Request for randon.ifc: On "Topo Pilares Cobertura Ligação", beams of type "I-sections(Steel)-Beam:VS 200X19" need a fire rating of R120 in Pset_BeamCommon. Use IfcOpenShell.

First a look at what the model holds.

```python
import ifcopenshell
import ifcopenshell.util.element

model = ifcopenshell.open("randon.ifc")
print(model.schema)
storey = next(s for s in model.by_type("IfcBuildingStorey") if s.Name == "Topo Pilares Cobertura Ligação")
beams = [e for e in ifcopenshell.util.element.get_decomposition(storey) if e.is_a("IfcBeam")]
seen = {}
for e in beams:
    element_type = ifcopenshell.util.element.get_type(e)
    key = (element_type.Name if element_type != e and element_type else None, ifcopenshell.util.element.get_pset(e, "Pset_BeamCommon", "FireRating"))
    seen[key] = seen.get(key, 0) + 1
for (name, value), count in sorted(seen.items(), key=str):
    print(count, "x", name, "|", value)
```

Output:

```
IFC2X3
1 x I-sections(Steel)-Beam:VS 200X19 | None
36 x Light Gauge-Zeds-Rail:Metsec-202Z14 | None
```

```python
import ifcopenshell
import ifcopenshell.api.pset
import ifcopenshell.util.element

model = ifcopenshell.open("randon.ifc")

storey = next(s for s in model.by_type("IfcBuildingStorey") if s.Name == "Topo Pilares Cobertura Ligação")
beams = [e for e in ifcopenshell.util.element.get_decomposition(storey) if e.is_a("IfcBeam")]

count = 0
for e in beams:
    element_type = ifcopenshell.util.element.get_type(e)
    if element_type in (None, e) or element_type.Name != "I-sections(Steel)-Beam:VS 200X19":
        continue
    # add_pset returns the element's existing set when there is one.
    pset = ifcopenshell.api.pset.add_pset(model, product=e, name="Pset_BeamCommon")
    ifcopenshell.api.pset.edit_pset(model, pset=pset, properties={"FireRating": "R120"})
    count += 1

print(count, "beams updated")

model.write("randon_updated.ifc")
```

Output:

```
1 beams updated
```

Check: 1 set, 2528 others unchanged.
